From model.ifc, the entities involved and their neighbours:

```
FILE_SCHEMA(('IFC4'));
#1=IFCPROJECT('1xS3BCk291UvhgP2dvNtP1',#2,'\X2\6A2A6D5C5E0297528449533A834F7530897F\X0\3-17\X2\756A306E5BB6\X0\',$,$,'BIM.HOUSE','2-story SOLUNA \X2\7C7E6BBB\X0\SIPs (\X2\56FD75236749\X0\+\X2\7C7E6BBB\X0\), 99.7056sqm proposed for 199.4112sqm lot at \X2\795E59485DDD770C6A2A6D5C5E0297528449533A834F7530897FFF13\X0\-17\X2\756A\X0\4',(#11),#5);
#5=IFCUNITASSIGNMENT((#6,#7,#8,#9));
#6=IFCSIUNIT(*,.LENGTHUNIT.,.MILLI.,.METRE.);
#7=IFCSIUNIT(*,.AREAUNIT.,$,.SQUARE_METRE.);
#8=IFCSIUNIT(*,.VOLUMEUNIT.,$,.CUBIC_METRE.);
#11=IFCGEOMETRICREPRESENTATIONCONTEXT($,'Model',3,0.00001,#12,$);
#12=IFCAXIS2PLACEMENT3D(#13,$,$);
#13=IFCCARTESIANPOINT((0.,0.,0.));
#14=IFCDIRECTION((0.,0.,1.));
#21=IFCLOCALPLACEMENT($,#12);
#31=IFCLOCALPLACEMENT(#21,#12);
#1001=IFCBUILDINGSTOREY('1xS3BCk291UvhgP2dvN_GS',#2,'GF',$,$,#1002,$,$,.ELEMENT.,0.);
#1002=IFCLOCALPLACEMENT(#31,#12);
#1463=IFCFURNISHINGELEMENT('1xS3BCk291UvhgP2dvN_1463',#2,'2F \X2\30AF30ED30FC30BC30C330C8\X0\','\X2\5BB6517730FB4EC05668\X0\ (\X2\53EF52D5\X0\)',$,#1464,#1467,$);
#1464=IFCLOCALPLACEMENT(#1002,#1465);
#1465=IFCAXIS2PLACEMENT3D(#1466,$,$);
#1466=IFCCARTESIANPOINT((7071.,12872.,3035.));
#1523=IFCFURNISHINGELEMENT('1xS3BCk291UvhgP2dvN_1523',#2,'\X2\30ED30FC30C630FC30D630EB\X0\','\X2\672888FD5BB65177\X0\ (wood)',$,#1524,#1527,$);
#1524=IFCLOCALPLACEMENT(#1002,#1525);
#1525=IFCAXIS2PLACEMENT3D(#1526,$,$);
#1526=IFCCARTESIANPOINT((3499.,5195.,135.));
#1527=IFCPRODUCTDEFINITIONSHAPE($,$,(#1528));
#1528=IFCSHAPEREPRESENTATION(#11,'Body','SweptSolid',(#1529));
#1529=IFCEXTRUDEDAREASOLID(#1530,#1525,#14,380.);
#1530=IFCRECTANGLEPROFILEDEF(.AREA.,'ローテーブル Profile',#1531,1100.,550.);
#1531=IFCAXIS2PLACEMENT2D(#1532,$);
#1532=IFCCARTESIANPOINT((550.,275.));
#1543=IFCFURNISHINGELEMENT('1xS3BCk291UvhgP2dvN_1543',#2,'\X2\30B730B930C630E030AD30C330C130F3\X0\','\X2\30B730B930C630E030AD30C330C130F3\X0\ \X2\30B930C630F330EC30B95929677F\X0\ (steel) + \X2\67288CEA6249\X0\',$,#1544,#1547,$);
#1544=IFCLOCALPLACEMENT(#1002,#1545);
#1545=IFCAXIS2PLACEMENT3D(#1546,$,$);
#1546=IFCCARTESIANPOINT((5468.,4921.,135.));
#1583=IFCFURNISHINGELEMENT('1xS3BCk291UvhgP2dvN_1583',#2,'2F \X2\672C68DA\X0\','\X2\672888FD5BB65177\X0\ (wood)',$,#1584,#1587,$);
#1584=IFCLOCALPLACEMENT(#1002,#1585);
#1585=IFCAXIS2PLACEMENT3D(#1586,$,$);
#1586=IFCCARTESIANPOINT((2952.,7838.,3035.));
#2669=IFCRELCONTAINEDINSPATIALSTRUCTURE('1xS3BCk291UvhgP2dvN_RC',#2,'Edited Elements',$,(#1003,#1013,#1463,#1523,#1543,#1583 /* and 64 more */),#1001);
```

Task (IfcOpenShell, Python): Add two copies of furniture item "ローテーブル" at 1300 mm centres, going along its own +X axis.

```python
import ifcopenshell
import ifcopenshell.api.geometry
import ifcopenshell.api.root
import ifcopenshell.util.element
import ifcopenshell.util.placement
import ifcopenshell.util.unit

model = ifcopenshell.open("model.ifc")
unit_scale = ifcopenshell.util.unit.calculate_unit_scale(model)


def reuse_history(source, copy):
    """copy_class also copies each property set's owner history, people and application; keep the originals."""
    for rel in copy.IsDefinedBy:
        if rel.is_a("IfcRelDefinesByProperties") and (history := rel.RelatingPropertyDefinition.OwnerHistory):
            rel.RelatingPropertyDefinition.OwnerHistory = source.OwnerHistory
            ifcopenshell.util.element.remove_deep2(model, history)


source = model.by_guid("1xS3BCk291UvhgP2dvN_1523")
base = ifcopenshell.util.placement.get_local_placement(source.ObjectPlacement)
step = base[:3, 0] * 1.3 / unit_scale

for i in range(1, 3):
    copy = ifcopenshell.api.root.copy_class(model, product=source)
    copy.Representation = ifcopenshell.util.element.copy_deep(
        model, source.Representation, exclude=["IfcGeometricRepresentationContext", "IfcRepresentationMap"]
    )
    reuse_history(source, copy)
    matrix = base.copy()
    matrix[:3, 3] += i * step
    print("added at", matrix[:3, 3].round(3) + 0.0)
    ifcopenshell.api.geometry.edit_object_placement(model, product=copy, matrix=matrix, is_si=False)

model.write("model-out.ifc")
```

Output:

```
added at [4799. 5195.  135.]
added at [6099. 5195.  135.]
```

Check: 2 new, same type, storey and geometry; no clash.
